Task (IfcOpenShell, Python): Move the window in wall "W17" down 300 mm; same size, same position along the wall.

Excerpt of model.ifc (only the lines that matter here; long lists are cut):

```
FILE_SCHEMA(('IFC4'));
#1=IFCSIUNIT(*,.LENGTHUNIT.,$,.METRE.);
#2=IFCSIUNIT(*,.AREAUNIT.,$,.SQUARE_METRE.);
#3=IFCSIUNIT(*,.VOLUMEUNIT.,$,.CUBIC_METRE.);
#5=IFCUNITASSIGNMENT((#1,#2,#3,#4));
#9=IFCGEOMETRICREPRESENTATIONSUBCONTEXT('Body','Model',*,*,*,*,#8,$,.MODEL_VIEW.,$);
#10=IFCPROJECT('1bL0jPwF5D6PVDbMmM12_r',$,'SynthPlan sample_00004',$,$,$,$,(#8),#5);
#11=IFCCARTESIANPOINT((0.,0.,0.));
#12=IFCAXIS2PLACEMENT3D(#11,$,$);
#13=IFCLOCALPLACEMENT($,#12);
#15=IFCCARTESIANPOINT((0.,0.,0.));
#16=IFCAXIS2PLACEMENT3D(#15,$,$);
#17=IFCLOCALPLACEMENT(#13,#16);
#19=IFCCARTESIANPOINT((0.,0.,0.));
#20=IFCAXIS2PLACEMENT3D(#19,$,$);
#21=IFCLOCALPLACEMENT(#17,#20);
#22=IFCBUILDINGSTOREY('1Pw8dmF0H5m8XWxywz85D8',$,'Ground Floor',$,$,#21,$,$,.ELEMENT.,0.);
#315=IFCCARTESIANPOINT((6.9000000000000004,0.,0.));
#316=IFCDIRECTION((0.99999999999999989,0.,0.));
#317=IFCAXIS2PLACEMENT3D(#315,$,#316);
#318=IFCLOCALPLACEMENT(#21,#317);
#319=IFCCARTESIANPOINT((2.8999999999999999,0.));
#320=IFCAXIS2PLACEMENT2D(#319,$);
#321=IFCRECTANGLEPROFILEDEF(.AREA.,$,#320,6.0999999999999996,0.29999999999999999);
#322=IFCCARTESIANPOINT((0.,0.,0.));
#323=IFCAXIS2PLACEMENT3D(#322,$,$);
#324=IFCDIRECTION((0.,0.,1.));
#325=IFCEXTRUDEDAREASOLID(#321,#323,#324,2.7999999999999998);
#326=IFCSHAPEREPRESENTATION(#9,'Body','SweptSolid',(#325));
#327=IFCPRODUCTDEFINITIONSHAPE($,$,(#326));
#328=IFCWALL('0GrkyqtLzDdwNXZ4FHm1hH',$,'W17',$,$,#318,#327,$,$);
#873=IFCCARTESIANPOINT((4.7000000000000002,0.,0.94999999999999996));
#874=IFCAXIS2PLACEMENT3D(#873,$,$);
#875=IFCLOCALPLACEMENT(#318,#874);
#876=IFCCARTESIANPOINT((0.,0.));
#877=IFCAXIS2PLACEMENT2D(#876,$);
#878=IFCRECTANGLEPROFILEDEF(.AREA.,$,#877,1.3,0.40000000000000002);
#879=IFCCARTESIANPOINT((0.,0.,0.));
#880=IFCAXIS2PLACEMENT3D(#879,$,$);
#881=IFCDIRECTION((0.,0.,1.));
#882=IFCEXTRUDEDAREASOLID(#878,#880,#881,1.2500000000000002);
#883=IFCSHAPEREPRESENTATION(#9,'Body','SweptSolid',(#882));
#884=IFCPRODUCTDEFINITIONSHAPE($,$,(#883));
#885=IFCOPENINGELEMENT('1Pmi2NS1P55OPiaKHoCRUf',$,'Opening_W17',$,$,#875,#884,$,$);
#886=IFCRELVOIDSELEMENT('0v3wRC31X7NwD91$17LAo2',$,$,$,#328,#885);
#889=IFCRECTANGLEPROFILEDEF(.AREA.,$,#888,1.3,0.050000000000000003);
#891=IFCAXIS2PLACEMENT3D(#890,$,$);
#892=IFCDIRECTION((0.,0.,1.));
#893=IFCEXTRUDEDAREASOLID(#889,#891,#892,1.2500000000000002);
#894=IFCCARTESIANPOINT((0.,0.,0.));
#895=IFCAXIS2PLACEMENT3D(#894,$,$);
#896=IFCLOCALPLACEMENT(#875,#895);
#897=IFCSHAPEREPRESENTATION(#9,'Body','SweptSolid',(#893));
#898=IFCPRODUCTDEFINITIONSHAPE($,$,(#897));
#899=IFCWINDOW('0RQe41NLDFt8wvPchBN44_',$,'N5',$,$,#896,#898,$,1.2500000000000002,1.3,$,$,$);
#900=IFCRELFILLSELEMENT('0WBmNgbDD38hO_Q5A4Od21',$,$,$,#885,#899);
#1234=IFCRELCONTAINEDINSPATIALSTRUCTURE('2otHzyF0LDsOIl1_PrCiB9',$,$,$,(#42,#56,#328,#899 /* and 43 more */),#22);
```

```python
import numpy as np
import ifcopenshell
import ifcopenshell.api.geometry
import ifcopenshell.util.placement
import ifcopenshell.util.unit

model = ifcopenshell.open("model.ifc")
unit_scale = ifcopenshell.util.unit.calculate_unit_scale(model)

window = model.by_guid("0RQe41NLDFt8wvPchBN44_")
opening = window.FillsVoids[0].RelatingOpeningElement
dz = -0.3

shift = np.array([0.0, 0.0, dz])
# The window is placed relative to its opening, so it follows when the opening moves.
matrix = ifcopenshell.util.placement.get_local_placement(opening.ObjectPlacement)
matrix[:3, 3] += shift
ifcopenshell.api.geometry.edit_object_placement(
    model, product=opening, matrix=matrix, is_si=False, should_transform_children=True
)

print(f"moved by {dz * unit_scale:+.3f} m")

model.write("model_v2.ifc")
```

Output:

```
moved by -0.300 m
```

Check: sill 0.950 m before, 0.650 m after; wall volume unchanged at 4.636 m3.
